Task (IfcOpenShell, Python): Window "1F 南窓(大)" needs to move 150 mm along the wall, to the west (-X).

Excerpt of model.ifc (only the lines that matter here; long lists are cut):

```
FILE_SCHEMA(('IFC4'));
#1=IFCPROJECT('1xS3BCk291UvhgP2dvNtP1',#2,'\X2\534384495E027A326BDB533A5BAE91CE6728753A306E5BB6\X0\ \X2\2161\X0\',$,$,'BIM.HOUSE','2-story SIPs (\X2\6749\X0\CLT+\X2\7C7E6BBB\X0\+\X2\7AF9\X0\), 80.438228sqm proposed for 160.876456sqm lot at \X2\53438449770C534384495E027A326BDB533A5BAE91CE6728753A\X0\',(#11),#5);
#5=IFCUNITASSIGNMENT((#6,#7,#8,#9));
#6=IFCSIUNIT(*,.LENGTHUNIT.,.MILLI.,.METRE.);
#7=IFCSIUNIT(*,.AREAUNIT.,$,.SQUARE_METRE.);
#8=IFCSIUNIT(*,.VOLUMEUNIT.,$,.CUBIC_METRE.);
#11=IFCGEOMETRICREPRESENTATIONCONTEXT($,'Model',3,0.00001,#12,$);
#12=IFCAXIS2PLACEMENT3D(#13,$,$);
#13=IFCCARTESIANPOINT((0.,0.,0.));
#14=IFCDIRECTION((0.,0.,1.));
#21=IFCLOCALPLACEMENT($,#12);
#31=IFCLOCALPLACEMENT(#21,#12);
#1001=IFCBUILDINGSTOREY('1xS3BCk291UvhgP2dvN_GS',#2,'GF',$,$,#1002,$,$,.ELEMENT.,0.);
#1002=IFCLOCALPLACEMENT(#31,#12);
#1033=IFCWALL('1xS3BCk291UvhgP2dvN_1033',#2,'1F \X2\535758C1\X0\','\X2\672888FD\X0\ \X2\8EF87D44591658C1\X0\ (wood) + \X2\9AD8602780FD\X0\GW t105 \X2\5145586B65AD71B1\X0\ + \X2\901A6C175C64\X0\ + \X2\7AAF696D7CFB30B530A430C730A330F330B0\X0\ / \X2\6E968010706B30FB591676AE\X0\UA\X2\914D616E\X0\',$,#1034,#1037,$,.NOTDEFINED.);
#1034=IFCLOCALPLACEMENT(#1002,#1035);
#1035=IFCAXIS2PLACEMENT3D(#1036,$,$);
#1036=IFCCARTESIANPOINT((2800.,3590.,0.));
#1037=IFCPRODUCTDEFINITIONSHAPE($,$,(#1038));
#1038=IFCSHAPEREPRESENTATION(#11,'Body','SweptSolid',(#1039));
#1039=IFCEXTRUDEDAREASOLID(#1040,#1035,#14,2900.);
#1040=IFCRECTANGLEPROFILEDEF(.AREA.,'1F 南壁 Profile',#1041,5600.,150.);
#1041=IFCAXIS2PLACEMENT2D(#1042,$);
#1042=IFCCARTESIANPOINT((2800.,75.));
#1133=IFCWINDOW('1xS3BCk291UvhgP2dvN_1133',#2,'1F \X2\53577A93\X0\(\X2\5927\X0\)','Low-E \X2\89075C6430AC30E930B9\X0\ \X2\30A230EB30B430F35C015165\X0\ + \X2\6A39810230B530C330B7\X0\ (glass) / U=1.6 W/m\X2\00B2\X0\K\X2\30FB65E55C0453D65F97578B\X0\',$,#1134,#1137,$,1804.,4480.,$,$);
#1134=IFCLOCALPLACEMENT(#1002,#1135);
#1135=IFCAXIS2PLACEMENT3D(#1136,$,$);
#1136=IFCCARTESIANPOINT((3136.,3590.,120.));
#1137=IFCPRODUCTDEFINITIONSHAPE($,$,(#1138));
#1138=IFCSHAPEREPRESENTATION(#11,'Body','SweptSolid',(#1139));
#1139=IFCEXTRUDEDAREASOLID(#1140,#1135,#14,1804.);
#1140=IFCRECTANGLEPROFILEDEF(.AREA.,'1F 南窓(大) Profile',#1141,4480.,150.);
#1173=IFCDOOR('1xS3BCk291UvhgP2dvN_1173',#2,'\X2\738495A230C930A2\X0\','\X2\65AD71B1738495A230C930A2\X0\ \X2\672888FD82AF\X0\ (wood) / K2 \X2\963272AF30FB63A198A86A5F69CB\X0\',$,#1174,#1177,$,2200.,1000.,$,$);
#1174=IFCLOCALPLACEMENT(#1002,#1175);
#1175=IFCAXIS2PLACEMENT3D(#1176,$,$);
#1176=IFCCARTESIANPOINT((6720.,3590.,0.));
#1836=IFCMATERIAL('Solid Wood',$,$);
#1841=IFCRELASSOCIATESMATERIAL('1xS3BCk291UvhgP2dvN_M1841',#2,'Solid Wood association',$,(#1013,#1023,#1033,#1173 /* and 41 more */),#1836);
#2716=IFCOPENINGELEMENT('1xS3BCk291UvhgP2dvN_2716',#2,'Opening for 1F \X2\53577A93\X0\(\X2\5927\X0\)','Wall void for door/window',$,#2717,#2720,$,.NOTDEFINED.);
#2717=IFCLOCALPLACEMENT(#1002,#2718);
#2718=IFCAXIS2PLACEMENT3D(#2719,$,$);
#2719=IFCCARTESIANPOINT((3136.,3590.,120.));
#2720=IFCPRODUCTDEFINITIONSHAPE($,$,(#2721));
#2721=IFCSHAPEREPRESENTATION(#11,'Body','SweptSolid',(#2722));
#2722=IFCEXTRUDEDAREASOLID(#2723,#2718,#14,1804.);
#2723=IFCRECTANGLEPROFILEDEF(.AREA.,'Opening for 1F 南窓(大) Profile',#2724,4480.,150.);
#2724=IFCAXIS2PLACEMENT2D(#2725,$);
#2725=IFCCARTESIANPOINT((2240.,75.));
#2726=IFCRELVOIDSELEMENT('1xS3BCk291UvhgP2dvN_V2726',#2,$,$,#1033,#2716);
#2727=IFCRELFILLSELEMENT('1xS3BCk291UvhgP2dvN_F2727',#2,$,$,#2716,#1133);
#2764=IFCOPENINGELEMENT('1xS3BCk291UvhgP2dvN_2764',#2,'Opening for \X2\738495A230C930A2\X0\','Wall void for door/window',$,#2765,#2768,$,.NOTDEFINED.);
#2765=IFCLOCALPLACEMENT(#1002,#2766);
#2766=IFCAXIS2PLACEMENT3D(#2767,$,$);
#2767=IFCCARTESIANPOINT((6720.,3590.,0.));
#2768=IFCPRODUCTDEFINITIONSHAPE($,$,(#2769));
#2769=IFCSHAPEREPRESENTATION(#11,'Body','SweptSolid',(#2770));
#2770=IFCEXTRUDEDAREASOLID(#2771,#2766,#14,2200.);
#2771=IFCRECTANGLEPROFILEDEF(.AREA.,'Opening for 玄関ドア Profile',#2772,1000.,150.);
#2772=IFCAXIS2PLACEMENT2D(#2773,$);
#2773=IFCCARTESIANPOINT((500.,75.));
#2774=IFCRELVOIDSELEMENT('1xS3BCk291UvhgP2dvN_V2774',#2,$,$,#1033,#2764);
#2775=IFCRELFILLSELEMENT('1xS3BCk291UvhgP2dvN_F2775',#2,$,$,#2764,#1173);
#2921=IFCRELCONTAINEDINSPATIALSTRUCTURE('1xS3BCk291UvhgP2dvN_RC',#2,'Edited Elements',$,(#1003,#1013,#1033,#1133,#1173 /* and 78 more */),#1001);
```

```python
import ifcopenshell
import ifcopenshell.api.geometry
import ifcopenshell.util.placement
import ifcopenshell.util.unit

model = ifcopenshell.open("model.ifc")
unit_scale = ifcopenshell.util.unit.calculate_unit_scale(model)

window = model.by_guid("1xS3BCk291UvhgP2dvN_1133")
opening = window.FillsVoids[0].RelatingOpeningElement
wall = opening.VoidsElements[0].RelatingBuildingElement

wall_matrix = ifcopenshell.util.placement.get_local_placement(wall.ObjectPlacement)
shift = wall_matrix[:3, 0] * -0.15 / unit_scale
before = ifcopenshell.util.placement.get_local_placement(window.ObjectPlacement)[:3, 3].copy()

# The window is not placed relative to its opening, so move both.
for product in (opening, window):
    matrix = ifcopenshell.util.placement.get_local_placement(product.ObjectPlacement)
    matrix[:3, 3] += shift
    ifcopenshell.api.geometry.edit_object_placement(model, product=product, matrix=matrix, is_si=False)

after = ifcopenshell.util.placement.get_local_placement(window.ObjectPlacement)[:3, 3]
print("window moved by", (after - before).round(3) + 0.0)

model.write("model-out.ifc")
```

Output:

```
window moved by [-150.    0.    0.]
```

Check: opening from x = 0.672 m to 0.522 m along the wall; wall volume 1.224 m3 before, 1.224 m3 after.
